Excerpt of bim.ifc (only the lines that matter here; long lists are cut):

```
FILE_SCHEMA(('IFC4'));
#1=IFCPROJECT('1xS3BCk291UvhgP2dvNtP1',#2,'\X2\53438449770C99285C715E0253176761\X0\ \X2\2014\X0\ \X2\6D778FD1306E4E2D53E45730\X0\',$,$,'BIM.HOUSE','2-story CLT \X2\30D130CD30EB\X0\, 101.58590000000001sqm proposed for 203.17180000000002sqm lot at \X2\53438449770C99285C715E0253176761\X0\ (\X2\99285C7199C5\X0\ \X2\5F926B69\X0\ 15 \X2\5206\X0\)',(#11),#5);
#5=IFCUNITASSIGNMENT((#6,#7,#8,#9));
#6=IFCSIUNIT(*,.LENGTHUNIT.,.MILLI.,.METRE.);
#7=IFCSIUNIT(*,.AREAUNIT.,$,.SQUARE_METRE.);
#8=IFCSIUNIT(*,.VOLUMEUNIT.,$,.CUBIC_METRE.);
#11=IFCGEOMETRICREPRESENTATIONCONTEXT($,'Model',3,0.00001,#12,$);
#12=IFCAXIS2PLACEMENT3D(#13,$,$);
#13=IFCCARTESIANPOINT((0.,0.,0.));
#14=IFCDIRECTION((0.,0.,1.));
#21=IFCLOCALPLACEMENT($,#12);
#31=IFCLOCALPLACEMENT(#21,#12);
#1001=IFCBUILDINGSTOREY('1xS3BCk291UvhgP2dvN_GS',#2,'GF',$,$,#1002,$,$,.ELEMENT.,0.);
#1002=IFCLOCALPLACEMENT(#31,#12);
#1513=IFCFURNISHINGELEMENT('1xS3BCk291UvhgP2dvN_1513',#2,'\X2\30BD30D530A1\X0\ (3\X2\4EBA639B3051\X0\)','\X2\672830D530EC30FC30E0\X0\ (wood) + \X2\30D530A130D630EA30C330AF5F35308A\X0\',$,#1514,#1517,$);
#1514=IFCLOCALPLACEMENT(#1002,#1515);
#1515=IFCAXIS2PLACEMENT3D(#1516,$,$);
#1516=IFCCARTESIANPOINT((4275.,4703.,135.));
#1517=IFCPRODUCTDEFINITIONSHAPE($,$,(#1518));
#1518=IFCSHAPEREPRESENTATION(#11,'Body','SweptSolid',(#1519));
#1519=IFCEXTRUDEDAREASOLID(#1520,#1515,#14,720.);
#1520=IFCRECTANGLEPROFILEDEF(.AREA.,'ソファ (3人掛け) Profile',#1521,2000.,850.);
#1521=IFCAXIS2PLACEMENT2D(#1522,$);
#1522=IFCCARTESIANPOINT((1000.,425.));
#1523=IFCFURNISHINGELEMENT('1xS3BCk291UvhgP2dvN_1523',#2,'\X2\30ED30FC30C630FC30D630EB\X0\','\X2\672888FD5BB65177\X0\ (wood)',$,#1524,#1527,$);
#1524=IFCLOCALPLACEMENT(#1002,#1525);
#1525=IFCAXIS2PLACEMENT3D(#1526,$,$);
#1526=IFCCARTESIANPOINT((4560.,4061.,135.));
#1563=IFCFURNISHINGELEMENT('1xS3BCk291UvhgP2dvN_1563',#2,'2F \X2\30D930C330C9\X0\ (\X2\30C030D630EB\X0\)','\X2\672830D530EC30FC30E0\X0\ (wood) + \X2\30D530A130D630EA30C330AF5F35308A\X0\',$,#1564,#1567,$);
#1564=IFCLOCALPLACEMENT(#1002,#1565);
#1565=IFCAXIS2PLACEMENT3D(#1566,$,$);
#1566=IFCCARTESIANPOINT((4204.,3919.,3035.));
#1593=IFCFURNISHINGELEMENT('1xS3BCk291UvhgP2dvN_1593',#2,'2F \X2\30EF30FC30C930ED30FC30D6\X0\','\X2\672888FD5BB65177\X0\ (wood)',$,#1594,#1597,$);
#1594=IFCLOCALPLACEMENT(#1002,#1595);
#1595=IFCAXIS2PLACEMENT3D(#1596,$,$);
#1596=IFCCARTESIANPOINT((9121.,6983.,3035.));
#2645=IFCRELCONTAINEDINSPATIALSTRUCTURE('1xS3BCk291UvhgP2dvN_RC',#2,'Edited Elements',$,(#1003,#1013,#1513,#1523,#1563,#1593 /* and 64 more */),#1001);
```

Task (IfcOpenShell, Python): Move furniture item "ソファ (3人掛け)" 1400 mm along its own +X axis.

```python
import ifcopenshell
import ifcopenshell.api.geometry
import ifcopenshell.util.placement
import ifcopenshell.util.unit

model = ifcopenshell.open("bim.ifc")
unit_scale = ifcopenshell.util.unit.calculate_unit_scale(model)

item = model.by_id(1513)
matrix = ifcopenshell.util.placement.get_local_placement(item.ObjectPlacement)
matrix[:3, 3] += matrix[:3, 0] * 1.4 / unit_scale
ifcopenshell.api.geometry.edit_object_placement(model, product=item, matrix=matrix, is_si=False)

print(ifcopenshell.util.placement.get_local_placement(item.ObjectPlacement).round(3) + 0.0)

model.write("bim-out.ifc")
```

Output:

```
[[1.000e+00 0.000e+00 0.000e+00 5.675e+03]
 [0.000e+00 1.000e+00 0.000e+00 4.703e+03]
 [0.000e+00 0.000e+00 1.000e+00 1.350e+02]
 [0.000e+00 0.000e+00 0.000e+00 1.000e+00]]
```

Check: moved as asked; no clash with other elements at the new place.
